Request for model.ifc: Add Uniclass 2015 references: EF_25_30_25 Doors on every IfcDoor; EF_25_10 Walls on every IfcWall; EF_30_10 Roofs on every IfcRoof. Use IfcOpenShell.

First a look at what the model holds.

```python
import ifcopenshell

model = ifcopenshell.open("model.ifc")
print(model.schema)
print("classifications:", [c.Name for c in model.by_type("IfcClassification")])
for ifc_class in ("IfcDoor", "IfcRoof", "IfcStair", "IfcWall", "IfcWindow"):
    print(ifc_class, len(model.by_type(ifc_class)))
```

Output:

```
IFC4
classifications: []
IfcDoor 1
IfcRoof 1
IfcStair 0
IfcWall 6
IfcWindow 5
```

```python
import ifcopenshell
import ifcopenshell.api.classification

model = ifcopenshell.open("model.ifc")

system = ifcopenshell.api.classification.add_classification(model, classification="Uniclass 2015")

codes = {
    "IfcDoor": ("EF_25_30_25", "Doors"),
    "IfcWall": ("EF_25_10", "Walls"),
    "IfcRoof": ("EF_30_10", "Roofs"),
}
for ifc_class, (code, name) in codes.items():
    products = model.by_type(ifc_class)
    ifcopenshell.api.classification.add_reference(
        model, products=products, classification=system, identification=code, name=name
    )
    print(code, len(products))

model.write("model_edited.ifc")
```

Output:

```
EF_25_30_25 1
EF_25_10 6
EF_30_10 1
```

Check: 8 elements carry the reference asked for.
